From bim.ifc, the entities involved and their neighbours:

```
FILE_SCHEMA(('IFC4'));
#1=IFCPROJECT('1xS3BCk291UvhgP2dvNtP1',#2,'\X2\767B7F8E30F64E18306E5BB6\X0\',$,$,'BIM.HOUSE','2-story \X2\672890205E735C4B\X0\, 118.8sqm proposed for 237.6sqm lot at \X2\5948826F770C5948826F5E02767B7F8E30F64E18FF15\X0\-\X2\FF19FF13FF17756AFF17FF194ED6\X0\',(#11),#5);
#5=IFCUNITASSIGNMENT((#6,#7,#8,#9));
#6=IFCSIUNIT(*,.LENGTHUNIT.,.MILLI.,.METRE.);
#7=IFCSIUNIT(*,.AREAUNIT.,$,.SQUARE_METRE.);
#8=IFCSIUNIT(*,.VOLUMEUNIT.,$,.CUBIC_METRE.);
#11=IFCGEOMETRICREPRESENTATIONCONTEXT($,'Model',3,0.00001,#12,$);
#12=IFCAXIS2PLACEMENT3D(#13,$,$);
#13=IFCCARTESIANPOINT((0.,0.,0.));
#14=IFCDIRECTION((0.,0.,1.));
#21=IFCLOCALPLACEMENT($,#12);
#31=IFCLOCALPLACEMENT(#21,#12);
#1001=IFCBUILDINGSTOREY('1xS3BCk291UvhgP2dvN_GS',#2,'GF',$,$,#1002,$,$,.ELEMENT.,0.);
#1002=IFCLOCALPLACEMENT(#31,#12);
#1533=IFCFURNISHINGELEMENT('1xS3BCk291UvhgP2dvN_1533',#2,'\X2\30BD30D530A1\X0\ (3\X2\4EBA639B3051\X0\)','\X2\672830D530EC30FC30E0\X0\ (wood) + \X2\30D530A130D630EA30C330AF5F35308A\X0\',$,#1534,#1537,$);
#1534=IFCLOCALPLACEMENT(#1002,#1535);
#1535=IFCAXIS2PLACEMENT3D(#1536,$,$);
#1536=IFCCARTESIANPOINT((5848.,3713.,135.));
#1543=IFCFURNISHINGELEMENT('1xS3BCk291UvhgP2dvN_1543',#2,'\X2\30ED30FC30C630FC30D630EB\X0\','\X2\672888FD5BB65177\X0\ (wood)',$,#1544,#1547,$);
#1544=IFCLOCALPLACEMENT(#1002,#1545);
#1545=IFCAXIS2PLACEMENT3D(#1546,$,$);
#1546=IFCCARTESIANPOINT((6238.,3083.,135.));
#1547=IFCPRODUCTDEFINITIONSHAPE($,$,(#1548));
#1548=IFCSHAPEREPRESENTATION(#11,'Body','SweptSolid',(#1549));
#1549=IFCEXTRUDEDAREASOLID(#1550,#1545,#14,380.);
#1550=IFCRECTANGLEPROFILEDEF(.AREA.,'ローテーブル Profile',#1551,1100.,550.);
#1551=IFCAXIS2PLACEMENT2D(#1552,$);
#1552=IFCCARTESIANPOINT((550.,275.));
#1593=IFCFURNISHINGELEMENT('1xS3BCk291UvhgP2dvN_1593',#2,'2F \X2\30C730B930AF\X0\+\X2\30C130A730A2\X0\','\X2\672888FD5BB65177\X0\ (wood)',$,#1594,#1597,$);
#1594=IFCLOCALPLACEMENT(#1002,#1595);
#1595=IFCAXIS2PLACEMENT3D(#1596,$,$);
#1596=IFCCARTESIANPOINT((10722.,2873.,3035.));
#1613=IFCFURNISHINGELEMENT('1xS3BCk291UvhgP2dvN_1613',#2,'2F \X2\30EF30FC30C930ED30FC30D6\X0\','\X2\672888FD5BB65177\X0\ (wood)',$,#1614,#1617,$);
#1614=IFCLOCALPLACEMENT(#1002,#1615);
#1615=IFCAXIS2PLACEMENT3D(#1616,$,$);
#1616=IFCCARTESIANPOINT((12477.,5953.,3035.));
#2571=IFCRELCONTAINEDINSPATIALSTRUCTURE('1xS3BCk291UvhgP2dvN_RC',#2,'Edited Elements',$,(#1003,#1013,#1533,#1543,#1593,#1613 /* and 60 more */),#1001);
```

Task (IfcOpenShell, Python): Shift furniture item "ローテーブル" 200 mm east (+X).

```python
import ifcopenshell
import ifcopenshell.api.geometry
import ifcopenshell.util.placement
import ifcopenshell.util.unit

model = ifcopenshell.open("bim.ifc")
unit_scale = ifcopenshell.util.unit.calculate_unit_scale(model)

item = model.by_id(1543)
matrix = ifcopenshell.util.placement.get_local_placement(item.ObjectPlacement)
matrix[0, 3] += 0.2 / unit_scale
ifcopenshell.api.geometry.edit_object_placement(model, product=item, matrix=matrix, is_si=False)

print(ifcopenshell.util.placement.get_local_placement(item.ObjectPlacement).round(3) + 0.0)

model.write("bim_edited.ifc")
```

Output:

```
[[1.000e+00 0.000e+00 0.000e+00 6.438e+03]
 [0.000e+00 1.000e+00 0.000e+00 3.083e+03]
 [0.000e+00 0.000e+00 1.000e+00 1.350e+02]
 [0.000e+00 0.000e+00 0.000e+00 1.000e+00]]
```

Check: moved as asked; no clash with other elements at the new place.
